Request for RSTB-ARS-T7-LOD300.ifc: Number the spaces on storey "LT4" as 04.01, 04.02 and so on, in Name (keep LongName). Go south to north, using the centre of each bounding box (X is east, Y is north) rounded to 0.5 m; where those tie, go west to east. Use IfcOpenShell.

First a look at what the model holds.

```python
import ifcopenshell
import ifcopenshell.util.element
import ifcopenshell.util.placement

model = ifcopenshell.open("RSTB-ARS-T7-LOD300.ifc")
print(model.schema)
storey = next(s for s in model.by_type("IfcBuildingStorey") if s.Name == "LT4")
spaces = [e for e in ifcopenshell.util.element.get_decomposition(storey) if e.is_a("IfcSpace")]
for e in sorted(spaces, key=lambda e: e.id()):
    origin = ifcopenshell.util.placement.get_local_placement(e.ObjectPlacement)[:3, 3]
    print(e.id(), e.Name, e.LongName, origin.round(2) + 0.0, sep=" | ")
```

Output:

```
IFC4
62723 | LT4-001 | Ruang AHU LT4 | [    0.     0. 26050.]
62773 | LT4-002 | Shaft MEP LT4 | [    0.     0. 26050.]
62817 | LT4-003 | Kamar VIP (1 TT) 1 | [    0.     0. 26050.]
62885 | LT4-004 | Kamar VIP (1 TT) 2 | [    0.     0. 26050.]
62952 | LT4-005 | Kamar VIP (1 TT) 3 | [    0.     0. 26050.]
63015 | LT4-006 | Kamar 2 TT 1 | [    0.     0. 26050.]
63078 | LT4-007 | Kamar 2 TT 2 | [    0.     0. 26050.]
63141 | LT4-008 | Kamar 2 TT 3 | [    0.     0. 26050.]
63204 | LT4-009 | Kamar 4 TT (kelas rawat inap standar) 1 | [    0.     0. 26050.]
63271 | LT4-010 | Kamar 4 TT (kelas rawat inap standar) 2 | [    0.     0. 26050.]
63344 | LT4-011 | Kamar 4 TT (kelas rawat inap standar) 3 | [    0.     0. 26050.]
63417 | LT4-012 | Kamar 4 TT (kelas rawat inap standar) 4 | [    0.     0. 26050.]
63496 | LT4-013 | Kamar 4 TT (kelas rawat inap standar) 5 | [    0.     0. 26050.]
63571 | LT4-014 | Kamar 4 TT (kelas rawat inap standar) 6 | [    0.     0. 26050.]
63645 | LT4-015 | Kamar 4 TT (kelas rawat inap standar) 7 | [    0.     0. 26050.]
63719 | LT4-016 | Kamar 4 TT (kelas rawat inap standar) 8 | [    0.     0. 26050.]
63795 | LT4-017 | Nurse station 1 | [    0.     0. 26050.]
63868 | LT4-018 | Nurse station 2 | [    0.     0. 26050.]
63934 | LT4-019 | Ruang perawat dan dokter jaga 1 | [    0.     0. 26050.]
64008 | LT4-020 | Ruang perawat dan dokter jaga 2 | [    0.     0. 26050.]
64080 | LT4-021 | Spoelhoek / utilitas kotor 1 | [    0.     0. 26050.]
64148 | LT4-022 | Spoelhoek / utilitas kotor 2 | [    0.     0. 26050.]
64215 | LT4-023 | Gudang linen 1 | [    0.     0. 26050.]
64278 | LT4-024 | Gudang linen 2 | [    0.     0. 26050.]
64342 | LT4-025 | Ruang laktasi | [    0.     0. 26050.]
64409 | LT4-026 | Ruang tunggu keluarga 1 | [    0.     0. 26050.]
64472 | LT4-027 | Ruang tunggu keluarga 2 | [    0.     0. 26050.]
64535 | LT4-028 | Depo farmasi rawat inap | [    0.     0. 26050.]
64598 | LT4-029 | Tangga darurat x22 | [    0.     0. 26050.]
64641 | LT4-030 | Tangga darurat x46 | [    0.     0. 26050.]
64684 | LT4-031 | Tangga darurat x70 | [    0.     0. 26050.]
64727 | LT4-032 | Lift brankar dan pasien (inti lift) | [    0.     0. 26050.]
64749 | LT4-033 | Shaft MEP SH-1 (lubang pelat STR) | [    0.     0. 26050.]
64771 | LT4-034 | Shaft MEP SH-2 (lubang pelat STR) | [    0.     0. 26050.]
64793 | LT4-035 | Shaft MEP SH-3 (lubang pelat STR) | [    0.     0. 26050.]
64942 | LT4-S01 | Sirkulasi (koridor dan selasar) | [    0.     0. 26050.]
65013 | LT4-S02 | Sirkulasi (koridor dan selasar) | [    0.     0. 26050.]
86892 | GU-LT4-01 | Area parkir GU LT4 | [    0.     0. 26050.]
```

```python
import ifcopenshell
import ifcopenshell.geom
import ifcopenshell.util.element
import ifcopenshell.util.shape

model = ifcopenshell.open("RSTB-ARS-T7-LOD300.ifc")
settings = ifcopenshell.geom.settings()
settings.set("use-world-coords", True)


def centre(element):
    shape = ifcopenshell.geom.create_shape(settings, element)
    return ifcopenshell.util.shape.get_bbox_centroid(shape.geometry)


storey = next(s for s in model.by_type("IfcBuildingStorey") if s.Name == "LT4")
spaces = [e for e in ifcopenshell.util.element.get_decomposition(storey) if e.is_a("IfcSpace")]

# Insertion points can sit at a corner or the storey origin, so sort by the geometry (in metres).
centres = {e: centre(e) for e in spaces}
spaces.sort(key=lambda e: (round(centres[e][1] / 0.5), centres[e][0]))

for i, e in enumerate(spaces, start=1):
    number = f"04.{i:02d}"
    e.Name = number
    print(e.id(), number)

model.write("RSTB-ARS-T7-LOD300-out.ifc")
```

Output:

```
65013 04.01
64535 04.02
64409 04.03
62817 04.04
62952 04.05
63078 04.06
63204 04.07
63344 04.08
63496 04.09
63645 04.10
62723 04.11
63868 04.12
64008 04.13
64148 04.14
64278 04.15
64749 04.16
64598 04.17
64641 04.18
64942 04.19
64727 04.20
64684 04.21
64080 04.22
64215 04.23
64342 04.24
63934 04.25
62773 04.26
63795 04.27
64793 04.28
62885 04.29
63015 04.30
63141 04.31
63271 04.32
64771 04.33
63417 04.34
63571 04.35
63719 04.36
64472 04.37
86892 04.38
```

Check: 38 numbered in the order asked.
